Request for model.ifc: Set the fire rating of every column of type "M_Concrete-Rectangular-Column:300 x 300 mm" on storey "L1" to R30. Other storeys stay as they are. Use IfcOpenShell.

First a look at what the model holds.

```python
import ifcopenshell
import ifcopenshell.util.element

model = ifcopenshell.open("model.ifc")
print(model.schema)
storey = next(s for s in model.by_type("IfcBuildingStorey") if s.Name == "L1")
columns = [e for e in ifcopenshell.util.element.get_decomposition(storey) if e.is_a("IfcColumn")]
seen = {}
for e in columns:
    element_type = ifcopenshell.util.element.get_type(e)
    key = (element_type.Name if element_type != e and element_type else None, ifcopenshell.util.element.get_pset(e, "Pset_ColumnCommon", "FireRating"))
    seen[key] = seen.get(key, 0) + 1
for (name, value), count in sorted(seen.items(), key=str):
    print(count, "x", name, "|", value)
```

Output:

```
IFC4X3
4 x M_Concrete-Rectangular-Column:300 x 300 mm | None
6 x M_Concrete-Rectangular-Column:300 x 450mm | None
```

```python
import ifcopenshell
import ifcopenshell.api.pset
import ifcopenshell.util.element

model = ifcopenshell.open("model.ifc")

storey = next(s for s in model.by_type("IfcBuildingStorey") if s.Name == "L1")
columns = [e for e in ifcopenshell.util.element.get_decomposition(storey) if e.is_a("IfcColumn")]

count = 0
for e in columns:
    element_type = ifcopenshell.util.element.get_type(e)
    if element_type in (None, e) or element_type.Name != "M_Concrete-Rectangular-Column:300 x 300 mm":
        continue
    # add_pset returns the element's existing set when there is one.
    pset = ifcopenshell.api.pset.add_pset(model, product=e, name="Pset_ColumnCommon")
    ifcopenshell.api.pset.edit_pset(model, pset=pset, properties={"FireRating": "R30"})
    count += 1

print(count, "columns updated")

model.write("model_updated.ifc")
```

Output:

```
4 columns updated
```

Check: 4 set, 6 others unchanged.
